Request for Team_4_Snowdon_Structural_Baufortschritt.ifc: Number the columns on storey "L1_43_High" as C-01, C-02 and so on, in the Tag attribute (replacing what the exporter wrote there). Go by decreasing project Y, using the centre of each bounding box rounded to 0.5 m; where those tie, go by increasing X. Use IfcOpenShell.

First a look at what the model holds.

```python
import ifcopenshell
import ifcopenshell.util.element
import ifcopenshell.util.placement

model = ifcopenshell.open("Team_4_Snowdon_Structural_Baufortschritt.ifc")
print(model.schema)
storey = next(s for s in model.by_type("IfcBuildingStorey") if s.Name == "L1_43_High")
columns = [e for e in ifcopenshell.util.element.get_decomposition(storey) if e.is_a("IfcColumn")]
for e in sorted(columns, key=lambda e: e.id()):
    origin = ifcopenshell.util.placement.get_local_placement(e.ObjectPlacement)[:3, 3]
    print(e.id(), e.Tag, e.Name, origin.round(2) + 0.0, sep=" | ")
```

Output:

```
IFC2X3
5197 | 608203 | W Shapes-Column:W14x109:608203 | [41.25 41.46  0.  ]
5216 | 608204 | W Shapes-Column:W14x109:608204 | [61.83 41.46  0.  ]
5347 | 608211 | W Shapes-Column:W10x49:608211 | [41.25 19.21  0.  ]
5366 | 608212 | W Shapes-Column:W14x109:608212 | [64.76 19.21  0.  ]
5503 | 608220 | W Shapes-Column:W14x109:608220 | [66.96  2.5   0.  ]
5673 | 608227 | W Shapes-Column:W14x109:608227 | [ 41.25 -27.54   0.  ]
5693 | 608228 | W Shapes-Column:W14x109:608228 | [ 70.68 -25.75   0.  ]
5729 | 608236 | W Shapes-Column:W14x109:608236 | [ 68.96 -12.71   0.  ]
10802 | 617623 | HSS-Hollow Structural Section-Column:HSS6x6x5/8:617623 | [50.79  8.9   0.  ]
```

```python
import ifcopenshell
import ifcopenshell.geom
import ifcopenshell.util.element
import ifcopenshell.util.shape

model = ifcopenshell.open("Team_4_Snowdon_Structural_Baufortschritt.ifc")
settings = ifcopenshell.geom.settings()
settings.set("use-world-coords", True)


def centre(element):
    shape = ifcopenshell.geom.create_shape(settings, element)
    return ifcopenshell.util.shape.get_bbox_centroid(shape.geometry)


storey = next(s for s in model.by_type("IfcBuildingStorey") if s.Name == "L1_43_High")
columns = [e for e in ifcopenshell.util.element.get_decomposition(storey) if e.is_a("IfcColumn")]

# Insertion points can sit at a corner or the storey origin, so sort by the geometry (in metres).
centres = {e: centre(e) for e in columns}
columns.sort(key=lambda e: (-round(centres[e][1] / 0.5), centres[e][0]))

for i, e in enumerate(columns, start=1):
    number = f"C-{i:02d}"
    e.Tag = number
    print(e.id(), number)

model.write("Team_4_Snowdon_Structural_Baufortschritt-out.ifc")
```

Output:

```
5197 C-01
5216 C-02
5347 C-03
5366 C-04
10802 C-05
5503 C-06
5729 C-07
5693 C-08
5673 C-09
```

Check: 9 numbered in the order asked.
